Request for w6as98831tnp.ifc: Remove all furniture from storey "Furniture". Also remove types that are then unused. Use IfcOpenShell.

First a look at what the model holds.

```python
import ifcopenshell
import ifcopenshell.util.element

model = ifcopenshell.open("w6as98831tnp.ifc")
print(model.schema)
storey = next(s for s in model.by_type("IfcBuildingStorey") if s.Name == "Furniture")
furniture = [e for e in ifcopenshell.util.element.get_decomposition(storey) if e.is_a("IfcFurnishingElement")]
seen = {}
for e in furniture:
    element_type = ifcopenshell.util.element.get_type(e)
    name = element_type.Name if element_type not in (None, e) else None
    seen[name] = seen.get(name, 0) + 1
for name, count in sorted(seen.items(), key=str):
    print(count, "x", name)
```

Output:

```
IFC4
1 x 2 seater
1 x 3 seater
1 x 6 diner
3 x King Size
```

```python
import ifcopenshell
import ifcopenshell.api.root
import ifcopenshell.util.element

model = ifcopenshell.open("w6as98831tnp.ifc")

storey = next(s for s in model.by_type("IfcBuildingStorey") if s.Name == "Furniture")
furniture = [e for e in ifcopenshell.util.element.get_decomposition(storey) if e.is_a("IfcFurnishingElement")]
types = {ifcopenshell.util.element.get_type(e) for e in furniture} - {None, *furniture}

for e in furniture:
    ifcopenshell.api.root.remove_product(model, product=e)
print(len(furniture), "removed")

unused = [t for t in types if not ifcopenshell.util.element.get_types(t)]
for t in unused:
    ifcopenshell.api.root.remove_product(model, product=t)
print(len(unused), "unused types removed")

model.write("w6as98831tnp-out.ifc")
```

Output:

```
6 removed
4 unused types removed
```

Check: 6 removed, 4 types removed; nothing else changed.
